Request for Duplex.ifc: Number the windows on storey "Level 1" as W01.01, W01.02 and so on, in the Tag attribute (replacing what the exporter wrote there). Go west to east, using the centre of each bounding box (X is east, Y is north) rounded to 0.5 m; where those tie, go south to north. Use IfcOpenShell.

First a look at what the model holds.

```python
import ifcopenshell
import ifcopenshell.util.element
import ifcopenshell.util.placement

model = ifcopenshell.open("Duplex.ifc")
print(model.schema)
storey = next(s for s in model.by_type("IfcBuildingStorey") if s.Name == "Level 1")
windows = [e for e in ifcopenshell.util.element.get_decomposition(storey) if e.is_a("IfcWindow")]
for e in sorted(windows, key=lambda e: e.id()):
    origin = ifcopenshell.util.placement.get_local_placement(e.ObjectPlacement)[:3, 3]
    print(e.id(), e.Tag, e.Name, origin.round(2) + 0.0, sep=" | ")
```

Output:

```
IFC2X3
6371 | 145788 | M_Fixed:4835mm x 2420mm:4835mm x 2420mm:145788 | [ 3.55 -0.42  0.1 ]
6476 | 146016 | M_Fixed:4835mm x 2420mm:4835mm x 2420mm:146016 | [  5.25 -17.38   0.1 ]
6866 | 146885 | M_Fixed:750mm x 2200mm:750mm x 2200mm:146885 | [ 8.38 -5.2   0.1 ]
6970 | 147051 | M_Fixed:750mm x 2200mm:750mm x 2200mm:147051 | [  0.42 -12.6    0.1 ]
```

```python
import ifcopenshell
import ifcopenshell.geom
import ifcopenshell.util.element
import ifcopenshell.util.shape

model = ifcopenshell.open("Duplex.ifc")
settings = ifcopenshell.geom.settings()
settings.set("use-world-coords", True)


def centre(element):
    shape = ifcopenshell.geom.create_shape(settings, element)
    return ifcopenshell.util.shape.get_bbox_centroid(shape.geometry)


storey = next(s for s in model.by_type("IfcBuildingStorey") if s.Name == "Level 1")
windows = [e for e in ifcopenshell.util.element.get_decomposition(storey) if e.is_a("IfcWindow")]

# Insertion points can sit at a corner or the storey origin, so sort by the geometry (in metres).
centres = {e: centre(e) for e in windows}
windows.sort(key=lambda e: (round(centres[e][0] / 0.5), centres[e][1]))

for i, e in enumerate(windows, start=1):
    number = f"W01.{i:02d}"
    e.Tag = number
    print(e.id(), number)

model.write("Duplex-out.ifc")
```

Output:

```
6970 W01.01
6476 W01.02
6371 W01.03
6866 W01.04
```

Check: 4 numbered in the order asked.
